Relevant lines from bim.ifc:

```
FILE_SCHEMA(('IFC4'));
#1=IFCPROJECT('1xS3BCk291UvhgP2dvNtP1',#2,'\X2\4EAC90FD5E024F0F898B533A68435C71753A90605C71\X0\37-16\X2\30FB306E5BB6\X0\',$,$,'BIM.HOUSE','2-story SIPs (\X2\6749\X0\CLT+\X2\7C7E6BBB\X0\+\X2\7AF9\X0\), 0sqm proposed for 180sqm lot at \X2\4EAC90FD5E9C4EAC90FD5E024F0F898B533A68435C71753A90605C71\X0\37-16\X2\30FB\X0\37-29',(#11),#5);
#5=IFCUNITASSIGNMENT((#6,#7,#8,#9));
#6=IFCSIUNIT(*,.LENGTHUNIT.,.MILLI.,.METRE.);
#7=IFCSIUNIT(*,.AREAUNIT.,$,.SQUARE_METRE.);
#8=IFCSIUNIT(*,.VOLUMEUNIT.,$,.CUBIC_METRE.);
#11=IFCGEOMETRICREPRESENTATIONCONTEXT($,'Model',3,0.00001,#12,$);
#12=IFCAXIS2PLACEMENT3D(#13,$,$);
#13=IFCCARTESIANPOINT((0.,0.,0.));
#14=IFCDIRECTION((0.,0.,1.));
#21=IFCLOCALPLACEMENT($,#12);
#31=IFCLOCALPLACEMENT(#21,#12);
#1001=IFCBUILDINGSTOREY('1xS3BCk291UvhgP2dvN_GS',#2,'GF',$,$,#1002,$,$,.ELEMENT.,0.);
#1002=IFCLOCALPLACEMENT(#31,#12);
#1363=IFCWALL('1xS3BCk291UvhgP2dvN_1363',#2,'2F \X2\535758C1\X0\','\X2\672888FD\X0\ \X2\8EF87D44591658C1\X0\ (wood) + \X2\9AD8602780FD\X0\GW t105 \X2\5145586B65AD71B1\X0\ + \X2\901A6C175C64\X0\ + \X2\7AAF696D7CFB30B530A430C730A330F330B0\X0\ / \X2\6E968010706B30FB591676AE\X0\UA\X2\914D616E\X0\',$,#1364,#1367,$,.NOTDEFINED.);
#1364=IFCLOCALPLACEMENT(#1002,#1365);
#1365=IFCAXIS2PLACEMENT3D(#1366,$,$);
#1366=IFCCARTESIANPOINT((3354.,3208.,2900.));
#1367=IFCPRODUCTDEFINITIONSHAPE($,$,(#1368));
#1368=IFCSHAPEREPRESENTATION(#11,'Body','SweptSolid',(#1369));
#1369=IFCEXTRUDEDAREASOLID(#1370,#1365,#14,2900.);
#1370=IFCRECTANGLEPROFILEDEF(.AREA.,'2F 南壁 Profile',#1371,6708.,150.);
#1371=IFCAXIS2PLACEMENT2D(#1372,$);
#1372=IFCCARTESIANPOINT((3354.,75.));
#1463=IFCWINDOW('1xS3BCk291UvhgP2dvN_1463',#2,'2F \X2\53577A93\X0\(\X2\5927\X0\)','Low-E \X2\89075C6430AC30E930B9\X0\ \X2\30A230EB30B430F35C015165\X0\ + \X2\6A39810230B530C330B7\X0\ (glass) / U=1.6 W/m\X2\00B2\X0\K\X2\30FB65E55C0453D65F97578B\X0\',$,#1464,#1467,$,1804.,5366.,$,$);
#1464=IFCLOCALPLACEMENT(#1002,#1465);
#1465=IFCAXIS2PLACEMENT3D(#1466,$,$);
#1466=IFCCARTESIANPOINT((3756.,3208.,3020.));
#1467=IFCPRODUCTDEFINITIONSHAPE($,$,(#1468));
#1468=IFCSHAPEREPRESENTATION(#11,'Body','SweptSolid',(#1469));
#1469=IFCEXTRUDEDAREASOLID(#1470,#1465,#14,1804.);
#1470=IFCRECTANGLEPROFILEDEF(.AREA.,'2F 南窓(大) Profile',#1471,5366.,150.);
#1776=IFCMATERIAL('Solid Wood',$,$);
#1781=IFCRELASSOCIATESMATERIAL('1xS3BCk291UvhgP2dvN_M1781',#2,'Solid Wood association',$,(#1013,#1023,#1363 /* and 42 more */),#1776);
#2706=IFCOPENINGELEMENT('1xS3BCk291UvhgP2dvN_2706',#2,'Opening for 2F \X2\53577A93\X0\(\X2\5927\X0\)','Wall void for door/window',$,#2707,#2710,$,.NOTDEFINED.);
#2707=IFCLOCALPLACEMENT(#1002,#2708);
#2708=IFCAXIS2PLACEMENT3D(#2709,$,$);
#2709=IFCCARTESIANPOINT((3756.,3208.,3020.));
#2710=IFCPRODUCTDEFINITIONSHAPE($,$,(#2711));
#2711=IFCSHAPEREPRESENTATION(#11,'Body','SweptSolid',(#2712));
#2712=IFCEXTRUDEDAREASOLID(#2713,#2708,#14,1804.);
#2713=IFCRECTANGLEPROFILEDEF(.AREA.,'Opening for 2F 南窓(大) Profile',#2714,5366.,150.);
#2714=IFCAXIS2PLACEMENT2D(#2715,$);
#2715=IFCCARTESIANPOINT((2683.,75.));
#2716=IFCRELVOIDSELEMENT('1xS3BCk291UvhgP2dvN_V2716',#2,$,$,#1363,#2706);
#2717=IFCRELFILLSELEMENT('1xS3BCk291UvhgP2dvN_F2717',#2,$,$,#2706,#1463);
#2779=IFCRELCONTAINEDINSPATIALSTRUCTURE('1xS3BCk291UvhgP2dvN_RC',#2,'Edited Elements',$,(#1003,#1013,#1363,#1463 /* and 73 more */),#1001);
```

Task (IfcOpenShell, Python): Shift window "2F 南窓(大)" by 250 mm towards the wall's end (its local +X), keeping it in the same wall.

```python
import ifcopenshell
import ifcopenshell.api.geometry
import ifcopenshell.util.placement

model = ifcopenshell.open("bim.ifc")

window = model.by_guid("1xS3BCk291UvhgP2dvN_1463")
opening = window.FillsVoids[0].RelatingOpeningElement
wall = opening.VoidsElements[0].RelatingBuildingElement

wall_matrix = ifcopenshell.util.placement.get_local_placement(wall.ObjectPlacement)
shift = wall_matrix[:3, 0] * 250.0
before = ifcopenshell.util.placement.get_local_placement(window.ObjectPlacement)[:3, 3].copy()

# The window is not placed relative to its opening, so move both.
for product in (opening, window):
    matrix = ifcopenshell.util.placement.get_local_placement(product.ObjectPlacement)
    matrix[:3, 3] += shift
    ifcopenshell.api.geometry.edit_object_placement(model, product=product, matrix=matrix, is_si=False)

after = ifcopenshell.util.placement.get_local_placement(window.ObjectPlacement)[:3, 3]
print("window moved by", (after - before).round(3) + 0.0)

model.write("bim-out.ifc")
```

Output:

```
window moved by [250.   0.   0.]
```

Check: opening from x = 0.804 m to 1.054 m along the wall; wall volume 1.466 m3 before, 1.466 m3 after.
